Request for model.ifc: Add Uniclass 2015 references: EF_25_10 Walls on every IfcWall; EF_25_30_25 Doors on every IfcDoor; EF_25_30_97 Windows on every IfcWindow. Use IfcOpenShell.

First a look at what the model holds.

```python
import ifcopenshell

model = ifcopenshell.open("model.ifc")
print(model.schema)
print("classifications:", [c.Name for c in model.by_type("IfcClassification")])
for ifc_class in ("IfcDoor", "IfcRoof", "IfcStair", "IfcWall", "IfcWindow"):
    print(ifc_class, len(model.by_type(ifc_class)))
```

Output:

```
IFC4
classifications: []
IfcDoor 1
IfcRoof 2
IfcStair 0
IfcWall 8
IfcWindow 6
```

```python
import ifcopenshell
import ifcopenshell.api.classification

model = ifcopenshell.open("model.ifc")

system = ifcopenshell.api.classification.add_classification(model, classification="Uniclass 2015")

codes = {
    "IfcWall": ("EF_25_10", "Walls"),
    "IfcDoor": ("EF_25_30_25", "Doors"),
    "IfcWindow": ("EF_25_30_97", "Windows"),
}
for ifc_class, (code, name) in codes.items():
    products = model.by_type(ifc_class)
    ifcopenshell.api.classification.add_reference(
        model, products=products, classification=system, identification=code, name=name
    )
    print(code, len(products))

model.write("model_edited.ifc")
```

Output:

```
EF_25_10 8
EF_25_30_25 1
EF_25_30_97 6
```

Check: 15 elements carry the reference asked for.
